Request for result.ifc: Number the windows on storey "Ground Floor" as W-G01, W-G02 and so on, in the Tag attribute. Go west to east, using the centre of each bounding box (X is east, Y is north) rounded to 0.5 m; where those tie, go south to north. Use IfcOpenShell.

First a look at what the model holds.

```python
import ifcopenshell
import ifcopenshell.util.element
import ifcopenshell.util.placement

model = ifcopenshell.open("result.ifc")
print(model.schema)
storey = next(s for s in model.by_type("IfcBuildingStorey") if s.Name == "Ground Floor")
windows = [e for e in ifcopenshell.util.element.get_decomposition(storey) if e.is_a("IfcWindow")]
for e in sorted(windows, key=lambda e: e.id()):
    origin = ifcopenshell.util.placement.get_local_placement(e.ObjectPlacement)[:3, 3]
    print(e.id(), e.Tag, e.Name, origin.round(2) + 0.0, sep=" | ")
```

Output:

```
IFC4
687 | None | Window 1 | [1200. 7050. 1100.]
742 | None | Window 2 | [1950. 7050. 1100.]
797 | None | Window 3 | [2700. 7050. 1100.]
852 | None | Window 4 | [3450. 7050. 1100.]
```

```python
import ifcopenshell
import ifcopenshell.geom
import ifcopenshell.util.element
import ifcopenshell.util.shape

model = ifcopenshell.open("result.ifc")
settings = ifcopenshell.geom.settings()
settings.set("use-world-coords", True)


def centre(element):
    shape = ifcopenshell.geom.create_shape(settings, element)
    return ifcopenshell.util.shape.get_bbox_centroid(shape.geometry)


storey = next(s for s in model.by_type("IfcBuildingStorey") if s.Name == "Ground Floor")
windows = [e for e in ifcopenshell.util.element.get_decomposition(storey) if e.is_a("IfcWindow")]

# Insertion points can sit at a corner or the storey origin, so sort by the geometry (in metres).
centres = {e: centre(e) for e in windows}
windows.sort(key=lambda e: (round(centres[e][0] / 0.5), centres[e][1]))

for i, e in enumerate(windows, start=1):
    number = f"W-G{i:02d}"
    e.Tag = number
    print(e.id(), number)

model.write("result_rev.ifc")
```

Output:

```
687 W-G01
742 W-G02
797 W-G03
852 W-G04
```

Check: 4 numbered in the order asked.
